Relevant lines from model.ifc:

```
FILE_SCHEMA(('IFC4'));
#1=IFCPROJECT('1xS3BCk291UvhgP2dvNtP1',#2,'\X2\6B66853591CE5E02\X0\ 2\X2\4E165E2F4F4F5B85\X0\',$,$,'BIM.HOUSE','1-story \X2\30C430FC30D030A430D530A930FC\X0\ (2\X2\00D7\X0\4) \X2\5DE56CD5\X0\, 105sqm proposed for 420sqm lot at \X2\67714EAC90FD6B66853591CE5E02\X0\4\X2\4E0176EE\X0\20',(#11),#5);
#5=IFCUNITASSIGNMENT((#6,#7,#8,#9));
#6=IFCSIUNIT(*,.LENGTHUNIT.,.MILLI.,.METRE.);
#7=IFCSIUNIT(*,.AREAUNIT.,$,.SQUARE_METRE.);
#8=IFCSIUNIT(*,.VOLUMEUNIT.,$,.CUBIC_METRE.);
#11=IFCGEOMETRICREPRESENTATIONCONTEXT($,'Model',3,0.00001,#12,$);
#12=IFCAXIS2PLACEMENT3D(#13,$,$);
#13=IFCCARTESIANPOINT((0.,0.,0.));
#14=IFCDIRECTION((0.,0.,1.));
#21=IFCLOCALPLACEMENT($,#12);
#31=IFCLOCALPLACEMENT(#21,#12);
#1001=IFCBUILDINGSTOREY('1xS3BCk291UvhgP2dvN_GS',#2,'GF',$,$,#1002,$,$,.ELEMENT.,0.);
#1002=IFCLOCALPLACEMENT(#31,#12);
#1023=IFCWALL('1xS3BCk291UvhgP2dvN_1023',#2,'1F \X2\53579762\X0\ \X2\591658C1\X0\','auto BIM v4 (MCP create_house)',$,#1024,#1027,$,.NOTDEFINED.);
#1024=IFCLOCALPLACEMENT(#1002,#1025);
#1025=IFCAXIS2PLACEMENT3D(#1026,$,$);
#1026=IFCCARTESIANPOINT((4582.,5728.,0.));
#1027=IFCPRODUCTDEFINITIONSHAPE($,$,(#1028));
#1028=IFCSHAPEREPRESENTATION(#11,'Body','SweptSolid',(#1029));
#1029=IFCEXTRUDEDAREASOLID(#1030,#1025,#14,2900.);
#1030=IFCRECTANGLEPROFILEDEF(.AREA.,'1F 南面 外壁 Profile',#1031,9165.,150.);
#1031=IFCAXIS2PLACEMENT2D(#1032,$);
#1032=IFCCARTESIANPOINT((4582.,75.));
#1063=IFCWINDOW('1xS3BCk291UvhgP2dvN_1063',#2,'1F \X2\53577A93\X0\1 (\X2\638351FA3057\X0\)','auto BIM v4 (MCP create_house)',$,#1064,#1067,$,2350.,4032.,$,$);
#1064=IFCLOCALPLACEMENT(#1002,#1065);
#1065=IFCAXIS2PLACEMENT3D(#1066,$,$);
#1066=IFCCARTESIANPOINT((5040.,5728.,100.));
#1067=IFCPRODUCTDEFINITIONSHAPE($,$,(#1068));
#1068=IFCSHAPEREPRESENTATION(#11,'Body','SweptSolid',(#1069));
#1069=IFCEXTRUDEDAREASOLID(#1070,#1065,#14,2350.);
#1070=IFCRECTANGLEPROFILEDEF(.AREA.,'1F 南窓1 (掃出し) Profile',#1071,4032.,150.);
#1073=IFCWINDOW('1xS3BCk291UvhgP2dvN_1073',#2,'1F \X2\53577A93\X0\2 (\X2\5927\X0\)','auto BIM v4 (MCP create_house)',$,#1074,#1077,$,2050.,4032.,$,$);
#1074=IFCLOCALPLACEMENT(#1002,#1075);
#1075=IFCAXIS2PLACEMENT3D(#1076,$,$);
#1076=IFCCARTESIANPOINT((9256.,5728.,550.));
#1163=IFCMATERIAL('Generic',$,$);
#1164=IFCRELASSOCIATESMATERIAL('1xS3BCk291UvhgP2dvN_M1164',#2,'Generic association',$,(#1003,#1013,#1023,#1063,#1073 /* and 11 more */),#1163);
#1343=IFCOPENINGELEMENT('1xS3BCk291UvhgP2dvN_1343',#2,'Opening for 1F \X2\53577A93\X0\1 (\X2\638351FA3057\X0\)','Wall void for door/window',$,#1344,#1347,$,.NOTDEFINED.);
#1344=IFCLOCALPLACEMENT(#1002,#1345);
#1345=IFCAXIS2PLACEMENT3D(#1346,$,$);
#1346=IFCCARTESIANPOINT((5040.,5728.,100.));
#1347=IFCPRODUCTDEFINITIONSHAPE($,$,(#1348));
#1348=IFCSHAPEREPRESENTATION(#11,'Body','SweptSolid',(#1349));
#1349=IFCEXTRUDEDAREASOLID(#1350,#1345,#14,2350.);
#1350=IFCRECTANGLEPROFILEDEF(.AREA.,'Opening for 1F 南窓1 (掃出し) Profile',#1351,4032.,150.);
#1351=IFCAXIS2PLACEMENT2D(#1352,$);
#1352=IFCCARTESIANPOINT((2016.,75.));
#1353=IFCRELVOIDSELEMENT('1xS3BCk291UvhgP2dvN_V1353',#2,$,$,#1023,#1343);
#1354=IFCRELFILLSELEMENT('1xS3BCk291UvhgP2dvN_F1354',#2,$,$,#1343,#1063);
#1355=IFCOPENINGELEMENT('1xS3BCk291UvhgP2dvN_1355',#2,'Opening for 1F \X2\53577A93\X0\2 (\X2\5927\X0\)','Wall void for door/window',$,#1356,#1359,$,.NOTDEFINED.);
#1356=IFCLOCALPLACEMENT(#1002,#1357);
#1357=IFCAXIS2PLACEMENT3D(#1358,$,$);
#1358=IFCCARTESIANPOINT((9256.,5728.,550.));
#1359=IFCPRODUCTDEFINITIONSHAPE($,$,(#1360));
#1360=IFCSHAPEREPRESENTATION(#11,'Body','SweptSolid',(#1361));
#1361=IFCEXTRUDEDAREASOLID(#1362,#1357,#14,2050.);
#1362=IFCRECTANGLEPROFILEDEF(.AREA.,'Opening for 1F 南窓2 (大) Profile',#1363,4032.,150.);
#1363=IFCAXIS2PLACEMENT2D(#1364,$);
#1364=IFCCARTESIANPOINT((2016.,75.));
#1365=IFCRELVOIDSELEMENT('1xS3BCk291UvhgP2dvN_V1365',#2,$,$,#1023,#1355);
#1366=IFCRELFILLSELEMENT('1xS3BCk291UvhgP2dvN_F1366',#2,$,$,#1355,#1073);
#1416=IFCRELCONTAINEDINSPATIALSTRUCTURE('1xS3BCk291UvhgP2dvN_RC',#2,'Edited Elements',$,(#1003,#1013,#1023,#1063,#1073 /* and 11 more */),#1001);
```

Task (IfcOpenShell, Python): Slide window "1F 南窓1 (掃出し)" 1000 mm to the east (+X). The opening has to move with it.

```python
import ifcopenshell
import ifcopenshell.api.geometry
import ifcopenshell.util.placement
import ifcopenshell.util.unit

model = ifcopenshell.open("model.ifc")
unit_scale = ifcopenshell.util.unit.calculate_unit_scale(model)

window = model.by_id(1063)
opening = window.FillsVoids[0].RelatingOpeningElement
wall = opening.VoidsElements[0].RelatingBuildingElement

wall_matrix = ifcopenshell.util.placement.get_local_placement(wall.ObjectPlacement)
shift = wall_matrix[:3, 0] * 1 / unit_scale
before = ifcopenshell.util.placement.get_local_placement(window.ObjectPlacement)[:3, 3].copy()

# The window is not placed relative to its opening, so move both.
for product in (opening, window):
    matrix = ifcopenshell.util.placement.get_local_placement(product.ObjectPlacement)
    matrix[:3, 3] += shift
    ifcopenshell.api.geometry.edit_object_placement(model, product=product, matrix=matrix, is_si=False)

after = ifcopenshell.util.placement.get_local_placement(window.ObjectPlacement)[:3, 3]
print("window moved by", (after - before).round(3) + 0.0)

model.write("model_edited.ifc")
```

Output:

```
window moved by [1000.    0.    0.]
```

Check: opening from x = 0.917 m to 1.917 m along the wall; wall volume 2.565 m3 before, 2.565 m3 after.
